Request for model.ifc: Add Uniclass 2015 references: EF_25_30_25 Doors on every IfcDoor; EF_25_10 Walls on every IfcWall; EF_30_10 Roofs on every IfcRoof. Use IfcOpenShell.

First a look at what the model holds.

```python
import ifcopenshell

model = ifcopenshell.open("model.ifc")
print(model.schema)
print("classifications:", [c.Name for c in model.by_type("IfcClassification")])
for ifc_class in ("IfcDoor", "IfcRoof", "IfcStair", "IfcWall", "IfcWindow"):
    print(ifc_class, len(model.by_type(ifc_class)))
```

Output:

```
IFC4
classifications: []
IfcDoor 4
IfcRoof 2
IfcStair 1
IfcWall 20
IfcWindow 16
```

```python
import ifcopenshell
import ifcopenshell.api.classification

model = ifcopenshell.open("model.ifc")

system = ifcopenshell.api.classification.add_classification(model, classification="Uniclass 2015")

codes = {
    "IfcDoor": ("EF_25_30_25", "Doors"),
    "IfcWall": ("EF_25_10", "Walls"),
    "IfcRoof": ("EF_30_10", "Roofs"),
}
for ifc_class, (code, name) in codes.items():
    products = model.by_type(ifc_class)
    ifcopenshell.api.classification.add_reference(
        model, products=products, classification=system, identification=code, name=name
    )
    print(code, len(products))

model.write("model-out.ifc")
```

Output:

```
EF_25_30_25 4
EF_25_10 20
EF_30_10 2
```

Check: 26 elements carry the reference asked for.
